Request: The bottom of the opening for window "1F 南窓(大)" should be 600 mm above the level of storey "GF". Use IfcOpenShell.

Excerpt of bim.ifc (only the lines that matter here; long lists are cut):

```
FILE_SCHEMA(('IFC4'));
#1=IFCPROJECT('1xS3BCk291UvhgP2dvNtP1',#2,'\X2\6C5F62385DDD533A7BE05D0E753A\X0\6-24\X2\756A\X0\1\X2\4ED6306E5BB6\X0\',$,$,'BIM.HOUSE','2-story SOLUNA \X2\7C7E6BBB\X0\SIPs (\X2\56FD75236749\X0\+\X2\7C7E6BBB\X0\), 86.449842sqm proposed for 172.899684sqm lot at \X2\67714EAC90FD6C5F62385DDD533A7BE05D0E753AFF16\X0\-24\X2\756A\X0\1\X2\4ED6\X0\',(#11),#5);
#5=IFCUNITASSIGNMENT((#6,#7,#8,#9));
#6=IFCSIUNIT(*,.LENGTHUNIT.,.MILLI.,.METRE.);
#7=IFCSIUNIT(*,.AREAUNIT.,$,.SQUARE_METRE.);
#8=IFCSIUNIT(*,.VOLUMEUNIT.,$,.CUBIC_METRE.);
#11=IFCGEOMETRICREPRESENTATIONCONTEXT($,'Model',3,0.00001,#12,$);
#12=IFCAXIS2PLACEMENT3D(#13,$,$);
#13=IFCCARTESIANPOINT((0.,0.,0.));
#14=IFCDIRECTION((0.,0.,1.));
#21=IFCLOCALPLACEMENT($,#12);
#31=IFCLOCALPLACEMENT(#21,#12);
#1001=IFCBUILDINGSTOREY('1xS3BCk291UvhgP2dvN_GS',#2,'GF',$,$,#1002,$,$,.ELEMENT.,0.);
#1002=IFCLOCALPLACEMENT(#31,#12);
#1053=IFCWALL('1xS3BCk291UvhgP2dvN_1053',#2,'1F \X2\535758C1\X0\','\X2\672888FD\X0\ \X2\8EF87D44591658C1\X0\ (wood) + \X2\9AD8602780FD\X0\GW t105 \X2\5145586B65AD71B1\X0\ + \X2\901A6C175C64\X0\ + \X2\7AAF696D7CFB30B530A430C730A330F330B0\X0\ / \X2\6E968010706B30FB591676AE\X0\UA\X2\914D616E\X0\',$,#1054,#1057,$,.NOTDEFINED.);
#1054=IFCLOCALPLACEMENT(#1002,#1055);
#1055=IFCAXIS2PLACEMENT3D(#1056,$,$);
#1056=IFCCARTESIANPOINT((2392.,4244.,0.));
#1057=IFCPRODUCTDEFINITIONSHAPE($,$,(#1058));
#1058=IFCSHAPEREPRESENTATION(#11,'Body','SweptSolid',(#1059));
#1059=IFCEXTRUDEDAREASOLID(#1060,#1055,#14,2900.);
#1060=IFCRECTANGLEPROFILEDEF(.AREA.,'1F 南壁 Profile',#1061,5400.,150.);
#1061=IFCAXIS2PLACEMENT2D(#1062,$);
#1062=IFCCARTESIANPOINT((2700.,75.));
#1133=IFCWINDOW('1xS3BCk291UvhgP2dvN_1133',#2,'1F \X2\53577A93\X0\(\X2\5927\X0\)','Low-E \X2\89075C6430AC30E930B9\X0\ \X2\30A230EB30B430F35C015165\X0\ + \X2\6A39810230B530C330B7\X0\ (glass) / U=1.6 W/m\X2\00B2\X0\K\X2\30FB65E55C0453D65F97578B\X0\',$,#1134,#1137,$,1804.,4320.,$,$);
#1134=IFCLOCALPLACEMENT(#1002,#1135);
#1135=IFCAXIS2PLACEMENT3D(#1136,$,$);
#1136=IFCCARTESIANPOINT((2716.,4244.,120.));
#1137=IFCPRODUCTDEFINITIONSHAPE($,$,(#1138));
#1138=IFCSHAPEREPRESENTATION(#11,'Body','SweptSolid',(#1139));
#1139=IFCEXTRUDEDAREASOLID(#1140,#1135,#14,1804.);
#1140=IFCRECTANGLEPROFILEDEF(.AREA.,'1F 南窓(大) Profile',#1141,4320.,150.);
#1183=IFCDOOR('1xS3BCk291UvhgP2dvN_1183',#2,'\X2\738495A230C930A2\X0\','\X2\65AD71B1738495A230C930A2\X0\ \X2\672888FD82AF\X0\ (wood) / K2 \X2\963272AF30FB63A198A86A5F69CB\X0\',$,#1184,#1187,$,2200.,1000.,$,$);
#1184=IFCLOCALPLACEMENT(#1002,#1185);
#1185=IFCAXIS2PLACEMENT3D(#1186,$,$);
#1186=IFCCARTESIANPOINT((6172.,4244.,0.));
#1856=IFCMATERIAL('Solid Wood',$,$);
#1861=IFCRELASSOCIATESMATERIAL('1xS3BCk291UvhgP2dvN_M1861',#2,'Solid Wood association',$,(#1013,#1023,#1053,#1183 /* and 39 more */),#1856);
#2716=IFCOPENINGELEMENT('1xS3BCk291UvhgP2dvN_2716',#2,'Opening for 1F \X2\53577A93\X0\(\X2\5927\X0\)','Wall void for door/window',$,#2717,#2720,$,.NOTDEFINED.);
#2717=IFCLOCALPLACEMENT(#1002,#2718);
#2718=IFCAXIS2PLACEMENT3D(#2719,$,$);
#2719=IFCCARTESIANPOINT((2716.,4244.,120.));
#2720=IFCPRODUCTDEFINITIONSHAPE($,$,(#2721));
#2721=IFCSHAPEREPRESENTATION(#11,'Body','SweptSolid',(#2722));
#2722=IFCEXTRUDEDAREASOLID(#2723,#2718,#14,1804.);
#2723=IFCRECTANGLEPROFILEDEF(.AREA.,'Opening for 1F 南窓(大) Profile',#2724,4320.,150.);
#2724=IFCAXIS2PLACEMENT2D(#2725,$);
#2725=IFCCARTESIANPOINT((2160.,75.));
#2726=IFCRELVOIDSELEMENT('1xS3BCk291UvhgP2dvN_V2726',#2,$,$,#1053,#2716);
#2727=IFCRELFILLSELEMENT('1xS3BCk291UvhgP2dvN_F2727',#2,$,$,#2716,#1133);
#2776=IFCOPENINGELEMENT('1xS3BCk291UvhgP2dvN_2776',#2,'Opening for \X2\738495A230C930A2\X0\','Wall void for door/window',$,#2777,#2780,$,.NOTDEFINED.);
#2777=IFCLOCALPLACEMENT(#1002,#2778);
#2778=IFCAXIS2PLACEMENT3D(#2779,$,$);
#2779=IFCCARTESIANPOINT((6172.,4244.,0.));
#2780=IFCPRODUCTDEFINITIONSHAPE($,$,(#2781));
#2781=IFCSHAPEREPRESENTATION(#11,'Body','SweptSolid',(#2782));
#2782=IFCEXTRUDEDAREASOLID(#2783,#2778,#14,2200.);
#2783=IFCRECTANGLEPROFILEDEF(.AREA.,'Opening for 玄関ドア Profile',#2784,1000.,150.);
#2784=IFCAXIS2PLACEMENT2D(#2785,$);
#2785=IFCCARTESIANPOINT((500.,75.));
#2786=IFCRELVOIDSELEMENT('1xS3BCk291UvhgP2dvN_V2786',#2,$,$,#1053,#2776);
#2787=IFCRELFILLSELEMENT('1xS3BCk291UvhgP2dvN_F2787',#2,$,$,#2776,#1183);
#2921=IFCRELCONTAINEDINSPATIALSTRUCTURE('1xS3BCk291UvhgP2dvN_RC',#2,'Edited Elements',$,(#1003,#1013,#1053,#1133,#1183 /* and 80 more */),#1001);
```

```python
import numpy as np
import ifcopenshell
import ifcopenshell.api.geometry
import ifcopenshell.geom
import ifcopenshell.util.element
import ifcopenshell.util.placement
import ifcopenshell.util.shape
import ifcopenshell.util.unit

model = ifcopenshell.open("bim.ifc")
unit_scale = ifcopenshell.util.unit.calculate_unit_scale(model)

window = model.by_guid("1xS3BCk291UvhgP2dvN_1133")
opening = window.FillsVoids[0].RelatingOpeningElement
storey = ifcopenshell.util.element.get_container(window, ifc_class="IfcBuildingStorey")
level = ifcopenshell.util.placement.get_local_placement(storey.ObjectPlacement)[2, 3]

# The opening's origin need not be at the sill, so measure its lowest point.
shape = ifcopenshell.geom.create_shape(ifcopenshell.geom.settings(), opening)
bottom = ifcopenshell.util.shape.get_shape_bottom_elevation(shape, shape.geometry) / unit_scale
dz = level + 600.0 - bottom

shift = np.array([0.0, 0.0, dz])
# The window is not placed relative to its opening, so move both.
for product in (opening, window):
    matrix = ifcopenshell.util.placement.get_local_placement(product.ObjectPlacement)
    matrix[:3, 3] += shift
    ifcopenshell.api.geometry.edit_object_placement(model, product=product, matrix=matrix, is_si=False)

print(f"moved by {dz * unit_scale:+.3f} m")

model.write("bim_edited.ifc")
```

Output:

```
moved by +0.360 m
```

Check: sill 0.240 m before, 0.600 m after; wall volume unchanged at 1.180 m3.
